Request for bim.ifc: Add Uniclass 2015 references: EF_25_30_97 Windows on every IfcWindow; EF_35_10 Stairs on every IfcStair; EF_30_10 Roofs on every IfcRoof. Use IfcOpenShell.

First a look at what the model holds.

```python
import ifcopenshell

model = ifcopenshell.open("bim.ifc")
print(model.schema)
print("classifications:", [c.Name for c in model.by_type("IfcClassification")])
for ifc_class in ("IfcDoor", "IfcRoof", "IfcStair", "IfcWall", "IfcWindow"):
    print(ifc_class, len(model.by_type(ifc_class)))
```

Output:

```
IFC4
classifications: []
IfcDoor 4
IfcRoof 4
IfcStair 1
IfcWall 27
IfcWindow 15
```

```python
import ifcopenshell
import ifcopenshell.api.classification

model = ifcopenshell.open("bim.ifc")

system = ifcopenshell.api.classification.add_classification(model, classification="Uniclass 2015")

codes = {
    "IfcWindow": ("EF_25_30_97", "Windows"),
    "IfcStair": ("EF_35_10", "Stairs"),
    "IfcRoof": ("EF_30_10", "Roofs"),
}
for ifc_class, (code, name) in codes.items():
    products = model.by_type(ifc_class)
    ifcopenshell.api.classification.add_reference(
        model, products=products, classification=system, identification=code, name=name
    )
    print(code, len(products))

model.write("bim_updated.ifc")
```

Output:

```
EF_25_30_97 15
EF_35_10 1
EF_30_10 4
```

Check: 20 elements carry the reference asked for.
